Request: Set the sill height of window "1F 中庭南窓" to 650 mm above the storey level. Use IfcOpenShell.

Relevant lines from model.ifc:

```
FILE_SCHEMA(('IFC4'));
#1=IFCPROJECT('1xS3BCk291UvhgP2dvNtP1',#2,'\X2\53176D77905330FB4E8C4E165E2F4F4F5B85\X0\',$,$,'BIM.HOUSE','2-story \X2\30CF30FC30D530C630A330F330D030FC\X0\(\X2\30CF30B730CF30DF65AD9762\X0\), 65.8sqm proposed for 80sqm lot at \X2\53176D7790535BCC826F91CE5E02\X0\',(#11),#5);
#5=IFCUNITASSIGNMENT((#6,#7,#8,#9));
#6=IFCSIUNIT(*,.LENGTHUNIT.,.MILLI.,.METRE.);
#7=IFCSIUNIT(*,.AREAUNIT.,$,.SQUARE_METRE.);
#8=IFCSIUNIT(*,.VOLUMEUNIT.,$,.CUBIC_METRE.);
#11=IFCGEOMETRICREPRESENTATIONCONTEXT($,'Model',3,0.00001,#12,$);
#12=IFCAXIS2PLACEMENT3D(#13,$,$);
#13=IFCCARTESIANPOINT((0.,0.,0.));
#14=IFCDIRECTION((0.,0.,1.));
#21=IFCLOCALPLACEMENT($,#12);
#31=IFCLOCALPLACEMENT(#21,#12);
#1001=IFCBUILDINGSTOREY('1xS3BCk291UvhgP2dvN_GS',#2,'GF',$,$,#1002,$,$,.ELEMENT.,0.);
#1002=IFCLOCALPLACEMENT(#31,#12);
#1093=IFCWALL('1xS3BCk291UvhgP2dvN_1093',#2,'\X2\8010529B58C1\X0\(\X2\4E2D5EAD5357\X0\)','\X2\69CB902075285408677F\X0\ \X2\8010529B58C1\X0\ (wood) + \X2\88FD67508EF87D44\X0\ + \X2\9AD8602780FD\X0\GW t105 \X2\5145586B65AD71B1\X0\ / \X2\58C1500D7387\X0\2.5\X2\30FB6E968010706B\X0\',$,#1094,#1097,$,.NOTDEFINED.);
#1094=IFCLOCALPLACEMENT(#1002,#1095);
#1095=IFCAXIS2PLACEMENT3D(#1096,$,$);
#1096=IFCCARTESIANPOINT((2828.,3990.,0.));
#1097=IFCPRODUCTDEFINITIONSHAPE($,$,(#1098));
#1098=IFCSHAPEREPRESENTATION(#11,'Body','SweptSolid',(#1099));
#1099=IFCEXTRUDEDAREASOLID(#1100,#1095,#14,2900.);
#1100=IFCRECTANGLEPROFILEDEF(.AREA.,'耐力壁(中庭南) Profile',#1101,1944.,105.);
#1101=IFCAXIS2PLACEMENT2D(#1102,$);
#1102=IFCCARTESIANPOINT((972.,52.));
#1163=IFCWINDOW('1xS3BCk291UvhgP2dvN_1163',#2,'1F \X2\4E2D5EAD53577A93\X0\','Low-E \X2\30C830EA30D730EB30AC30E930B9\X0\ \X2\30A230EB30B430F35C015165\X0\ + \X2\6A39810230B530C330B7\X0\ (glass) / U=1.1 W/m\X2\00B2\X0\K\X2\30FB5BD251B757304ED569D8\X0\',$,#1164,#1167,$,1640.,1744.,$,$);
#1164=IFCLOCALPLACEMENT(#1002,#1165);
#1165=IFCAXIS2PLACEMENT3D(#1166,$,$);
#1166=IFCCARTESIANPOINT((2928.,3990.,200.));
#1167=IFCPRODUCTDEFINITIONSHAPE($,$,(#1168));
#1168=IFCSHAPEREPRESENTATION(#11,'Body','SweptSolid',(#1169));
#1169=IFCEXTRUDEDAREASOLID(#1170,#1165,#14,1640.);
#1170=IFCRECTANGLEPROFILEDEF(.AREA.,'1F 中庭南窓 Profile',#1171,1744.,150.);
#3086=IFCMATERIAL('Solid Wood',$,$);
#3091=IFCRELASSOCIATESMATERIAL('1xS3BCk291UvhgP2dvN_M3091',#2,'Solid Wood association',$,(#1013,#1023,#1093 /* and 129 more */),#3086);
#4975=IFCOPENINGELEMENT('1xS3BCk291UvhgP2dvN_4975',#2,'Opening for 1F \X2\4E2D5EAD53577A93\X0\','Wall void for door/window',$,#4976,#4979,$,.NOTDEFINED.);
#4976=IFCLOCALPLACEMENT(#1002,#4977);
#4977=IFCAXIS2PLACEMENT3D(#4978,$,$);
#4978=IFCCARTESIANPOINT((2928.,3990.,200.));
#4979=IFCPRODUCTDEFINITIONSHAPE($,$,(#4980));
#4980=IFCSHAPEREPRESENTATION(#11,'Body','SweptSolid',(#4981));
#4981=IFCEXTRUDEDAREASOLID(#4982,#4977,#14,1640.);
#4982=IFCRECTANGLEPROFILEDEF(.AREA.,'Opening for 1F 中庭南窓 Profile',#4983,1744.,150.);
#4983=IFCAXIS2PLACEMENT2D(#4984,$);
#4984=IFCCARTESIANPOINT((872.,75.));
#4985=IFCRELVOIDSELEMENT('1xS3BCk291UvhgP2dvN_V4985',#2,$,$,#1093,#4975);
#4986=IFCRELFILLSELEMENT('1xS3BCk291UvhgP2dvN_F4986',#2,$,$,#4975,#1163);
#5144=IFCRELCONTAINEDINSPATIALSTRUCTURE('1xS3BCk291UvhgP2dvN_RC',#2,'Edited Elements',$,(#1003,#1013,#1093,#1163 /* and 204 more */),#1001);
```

```python
import numpy as np
import ifcopenshell
import ifcopenshell.api.geometry
import ifcopenshell.geom
import ifcopenshell.util.element
import ifcopenshell.util.placement
import ifcopenshell.util.shape
import ifcopenshell.util.unit

model = ifcopenshell.open("model.ifc")
unit_scale = ifcopenshell.util.unit.calculate_unit_scale(model)

window = model.by_guid("1xS3BCk291UvhgP2dvN_1163")
opening = window.FillsVoids[0].RelatingOpeningElement
storey = ifcopenshell.util.element.get_container(window, ifc_class="IfcBuildingStorey")
level = ifcopenshell.util.placement.get_local_placement(storey.ObjectPlacement)[2, 3]

# The opening's origin need not be at the sill, so measure its lowest point.
shape = ifcopenshell.geom.create_shape(ifcopenshell.geom.settings(), opening)
bottom = ifcopenshell.util.shape.get_shape_bottom_elevation(shape, shape.geometry) / unit_scale
dz = level + 0.65 / unit_scale - bottom

shift = np.array([0.0, 0.0, dz])
# The window is not placed relative to its opening, so move both.
for product in (opening, window):
    matrix = ifcopenshell.util.placement.get_local_placement(product.ObjectPlacement)
    matrix[:3, 3] += shift
    ifcopenshell.api.geometry.edit_object_placement(model, product=product, matrix=matrix, is_si=False)

print(f"moved by {dz * unit_scale:+.3f} m")

model.write("model_updated.ifc")
```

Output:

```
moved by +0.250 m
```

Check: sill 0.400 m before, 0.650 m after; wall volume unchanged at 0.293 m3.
